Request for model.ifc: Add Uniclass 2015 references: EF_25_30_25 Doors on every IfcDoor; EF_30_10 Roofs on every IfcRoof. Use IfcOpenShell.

First a look at what the model holds.

```python
import ifcopenshell

model = ifcopenshell.open("model.ifc")
print(model.schema)
print("classifications:", [c.Name for c in model.by_type("IfcClassification")])
for ifc_class in ("IfcDoor", "IfcRoof", "IfcStair", "IfcWall", "IfcWindow"):
    print(ifc_class, len(model.by_type(ifc_class)))
```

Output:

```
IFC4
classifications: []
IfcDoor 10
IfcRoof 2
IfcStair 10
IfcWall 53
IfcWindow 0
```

```python
import ifcopenshell
import ifcopenshell.api.classification

model = ifcopenshell.open("model.ifc")

system = ifcopenshell.api.classification.add_classification(model, classification="Uniclass 2015")

codes = {
    "IfcDoor": ("EF_25_30_25", "Doors"),
    "IfcRoof": ("EF_30_10", "Roofs"),
}
for ifc_class, (code, name) in codes.items():
    products = model.by_type(ifc_class)
    ifcopenshell.api.classification.add_reference(
        model, products=products, classification=system, identification=code, name=name
    )
    print(code, len(products))

model.write("model-out.ifc")
```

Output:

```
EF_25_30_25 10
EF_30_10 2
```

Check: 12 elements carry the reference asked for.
